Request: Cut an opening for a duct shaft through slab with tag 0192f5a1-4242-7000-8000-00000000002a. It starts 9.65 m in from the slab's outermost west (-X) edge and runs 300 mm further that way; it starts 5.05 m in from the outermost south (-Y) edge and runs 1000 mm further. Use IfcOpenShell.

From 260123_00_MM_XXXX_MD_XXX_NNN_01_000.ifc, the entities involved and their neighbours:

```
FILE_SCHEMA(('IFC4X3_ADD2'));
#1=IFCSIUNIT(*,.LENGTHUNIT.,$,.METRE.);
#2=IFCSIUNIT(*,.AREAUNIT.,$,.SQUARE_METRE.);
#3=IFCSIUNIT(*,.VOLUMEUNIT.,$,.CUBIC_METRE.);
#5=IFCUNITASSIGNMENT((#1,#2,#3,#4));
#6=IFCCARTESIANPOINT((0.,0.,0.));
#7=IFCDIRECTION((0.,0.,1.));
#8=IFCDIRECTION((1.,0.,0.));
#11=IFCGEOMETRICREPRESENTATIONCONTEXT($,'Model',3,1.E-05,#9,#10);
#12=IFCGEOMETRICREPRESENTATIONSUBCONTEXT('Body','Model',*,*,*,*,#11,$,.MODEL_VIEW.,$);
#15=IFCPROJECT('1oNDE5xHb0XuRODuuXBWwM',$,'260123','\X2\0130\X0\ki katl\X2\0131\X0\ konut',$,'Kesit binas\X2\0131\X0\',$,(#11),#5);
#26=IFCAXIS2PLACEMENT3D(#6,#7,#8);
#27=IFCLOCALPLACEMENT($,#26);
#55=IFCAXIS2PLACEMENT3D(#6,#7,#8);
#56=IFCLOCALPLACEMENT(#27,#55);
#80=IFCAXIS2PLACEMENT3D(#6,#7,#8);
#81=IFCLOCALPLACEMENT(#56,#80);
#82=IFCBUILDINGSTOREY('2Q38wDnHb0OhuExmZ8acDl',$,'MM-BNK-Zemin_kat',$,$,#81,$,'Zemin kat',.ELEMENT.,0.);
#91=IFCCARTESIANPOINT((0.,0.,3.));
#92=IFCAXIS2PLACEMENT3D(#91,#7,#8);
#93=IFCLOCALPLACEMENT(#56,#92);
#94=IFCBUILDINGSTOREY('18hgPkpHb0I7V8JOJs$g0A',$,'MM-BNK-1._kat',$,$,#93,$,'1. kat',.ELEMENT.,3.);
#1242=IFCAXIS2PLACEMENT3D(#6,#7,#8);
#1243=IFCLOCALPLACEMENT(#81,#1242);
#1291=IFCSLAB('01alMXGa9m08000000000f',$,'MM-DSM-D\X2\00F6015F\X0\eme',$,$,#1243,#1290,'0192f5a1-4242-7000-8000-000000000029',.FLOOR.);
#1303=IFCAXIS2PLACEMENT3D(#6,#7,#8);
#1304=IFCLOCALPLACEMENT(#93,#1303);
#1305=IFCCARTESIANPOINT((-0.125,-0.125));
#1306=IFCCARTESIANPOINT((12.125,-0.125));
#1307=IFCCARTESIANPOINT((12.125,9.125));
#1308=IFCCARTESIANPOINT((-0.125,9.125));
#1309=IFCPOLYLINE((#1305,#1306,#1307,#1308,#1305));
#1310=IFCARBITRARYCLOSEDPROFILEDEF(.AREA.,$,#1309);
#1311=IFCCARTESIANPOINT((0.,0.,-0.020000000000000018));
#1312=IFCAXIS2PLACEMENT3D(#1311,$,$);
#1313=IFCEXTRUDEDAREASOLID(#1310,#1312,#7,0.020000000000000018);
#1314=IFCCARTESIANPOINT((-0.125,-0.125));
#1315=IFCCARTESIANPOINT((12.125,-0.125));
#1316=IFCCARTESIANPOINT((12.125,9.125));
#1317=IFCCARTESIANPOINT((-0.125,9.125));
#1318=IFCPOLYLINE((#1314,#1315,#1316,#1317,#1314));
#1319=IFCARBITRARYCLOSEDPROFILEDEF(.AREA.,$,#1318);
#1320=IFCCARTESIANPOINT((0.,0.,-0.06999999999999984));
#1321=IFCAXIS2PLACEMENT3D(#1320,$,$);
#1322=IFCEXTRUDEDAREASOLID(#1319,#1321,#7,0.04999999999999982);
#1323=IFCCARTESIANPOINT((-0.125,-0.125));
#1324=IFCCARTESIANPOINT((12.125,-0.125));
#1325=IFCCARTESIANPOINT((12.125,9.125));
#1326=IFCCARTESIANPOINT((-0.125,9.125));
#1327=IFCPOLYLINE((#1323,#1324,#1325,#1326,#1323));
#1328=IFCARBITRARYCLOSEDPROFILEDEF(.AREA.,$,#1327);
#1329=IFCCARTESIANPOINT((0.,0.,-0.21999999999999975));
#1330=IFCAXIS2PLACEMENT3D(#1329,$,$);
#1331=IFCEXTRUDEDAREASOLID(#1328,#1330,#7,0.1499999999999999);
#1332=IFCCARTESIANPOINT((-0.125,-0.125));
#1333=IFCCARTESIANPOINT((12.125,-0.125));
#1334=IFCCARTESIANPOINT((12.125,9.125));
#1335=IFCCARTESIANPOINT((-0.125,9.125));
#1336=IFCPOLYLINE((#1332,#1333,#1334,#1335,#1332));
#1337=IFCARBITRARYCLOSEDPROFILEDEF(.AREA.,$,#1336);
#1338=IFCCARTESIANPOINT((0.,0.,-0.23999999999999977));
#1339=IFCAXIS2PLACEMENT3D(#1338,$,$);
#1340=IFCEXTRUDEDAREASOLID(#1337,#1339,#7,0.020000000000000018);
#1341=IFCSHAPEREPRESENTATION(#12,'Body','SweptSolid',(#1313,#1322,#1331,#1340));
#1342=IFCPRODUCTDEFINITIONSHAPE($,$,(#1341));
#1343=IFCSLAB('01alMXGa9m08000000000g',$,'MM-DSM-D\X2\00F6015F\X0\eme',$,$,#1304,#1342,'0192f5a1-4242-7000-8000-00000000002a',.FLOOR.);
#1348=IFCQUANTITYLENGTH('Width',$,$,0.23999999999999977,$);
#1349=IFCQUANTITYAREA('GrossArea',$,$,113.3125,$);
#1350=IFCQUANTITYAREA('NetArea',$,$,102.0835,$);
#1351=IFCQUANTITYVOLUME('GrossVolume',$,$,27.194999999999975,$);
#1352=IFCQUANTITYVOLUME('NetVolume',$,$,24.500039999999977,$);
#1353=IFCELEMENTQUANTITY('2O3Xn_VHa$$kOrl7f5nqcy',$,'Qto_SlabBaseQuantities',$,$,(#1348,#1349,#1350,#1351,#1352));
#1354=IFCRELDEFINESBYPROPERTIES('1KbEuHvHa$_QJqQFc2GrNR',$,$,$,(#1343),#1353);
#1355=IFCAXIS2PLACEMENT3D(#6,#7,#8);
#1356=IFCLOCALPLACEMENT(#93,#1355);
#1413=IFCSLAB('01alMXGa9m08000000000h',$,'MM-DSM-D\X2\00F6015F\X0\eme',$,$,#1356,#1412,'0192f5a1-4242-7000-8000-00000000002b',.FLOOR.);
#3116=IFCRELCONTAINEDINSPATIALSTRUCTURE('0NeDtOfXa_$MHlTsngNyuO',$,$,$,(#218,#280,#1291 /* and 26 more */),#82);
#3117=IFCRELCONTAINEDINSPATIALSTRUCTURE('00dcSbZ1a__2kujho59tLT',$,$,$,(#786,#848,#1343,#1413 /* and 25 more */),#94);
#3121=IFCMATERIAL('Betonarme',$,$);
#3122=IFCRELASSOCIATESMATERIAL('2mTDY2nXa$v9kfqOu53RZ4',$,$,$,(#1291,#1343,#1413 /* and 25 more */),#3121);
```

```python
import numpy as np
import ifcopenshell
import ifcopenshell.api.feature
import ifcopenshell.api.geometry
import ifcopenshell.api.pset
import ifcopenshell.api.root
import ifcopenshell.geom
import ifcopenshell.util.element
import ifcopenshell.util.placement
import ifcopenshell.util.representation
import ifcopenshell.util.shape
import ifcopenshell.util.unit

model = ifcopenshell.open("260123_00_MM_XXXX_MD_XXX_NNN_01_000.ifc")
unit_scale = ifcopenshell.util.unit.calculate_unit_scale(model)
area_scale = ifcopenshell.util.unit.calculate_unit_scale(model, "AREAUNIT")
volume_scale = ifcopenshell.util.unit.calculate_unit_scale(model, "VOLUMEUNIT")
settings = ifcopenshell.geom.settings()


def volume(element):
    """Net volume in cubic metres, openings subtracted."""
    shape = ifcopenshell.geom.create_shape(settings, element)
    return ifcopenshell.util.shape.get_volume(shape.geometry)


slab = model.by_id(1343)
before = volume(slab)

# Extent in the slab's own axes, in metres. The edges named are its -X and -Y sides.
slab_shape = ifcopenshell.geom.create_shape(settings, slab)
vertices = ifcopenshell.util.shape.get_vertices(slab_shape.geometry)
x_min, y_min, bottom = vertices.min(axis=0)
top = vertices[:, 2].max()

opening = ifcopenshell.api.root.create_entity(model, ifc_class="IfcOpeningElement", name="Duct shaft opening", predefined_type="OPENING")
context = ifcopenshell.util.representation.get_context(model, "Model", "Body", "MODEL_VIEW")
width, depth = 0.3, 1
outline = [(0.0, 0.0), (width, 0.0), (width, depth), (0.0, depth), (0.0, 0.0)]
# Overshoot both faces by 50 mm so the cut is clean.
shape = ifcopenshell.api.geometry.add_slab_representation(
    model, context=context, depth=top - bottom + 0.1, polyline=outline
)
ifcopenshell.api.geometry.assign_representation(model, product=opening, representation=shape)

matrix = ifcopenshell.util.placement.get_local_placement(slab.ObjectPlacement)
matrix[:, 3] = matrix @ np.append(np.array([x_min + 9.65, y_min + 5.05, bottom - 0.05]) / unit_scale, 1.0)
ifcopenshell.api.geometry.edit_object_placement(model, product=opening, matrix=matrix, is_si=False)
ifcopenshell.api.feature.add_feature(model, feature=opening, element=slab)

after = volume(slab)

# Update the slab's stored quantities.
qto = model.by_id(ifcopenshell.util.element.get_pset(slab, "Qto_SlabBaseQuantities", should_inherit=False)["id"])
ifcopenshell.api.pset.edit_qto(model, qto=qto, properties={
    "NetArea": after / (top - bottom) / area_scale,
    "NetVolume": after / volume_scale,
})

print(f"slab volume {before:.3f} -> {after:.3f} m3")

model.write("260123_00_MM_XXXX_MD_XXX_NNN_01_000_updated.ifc")
```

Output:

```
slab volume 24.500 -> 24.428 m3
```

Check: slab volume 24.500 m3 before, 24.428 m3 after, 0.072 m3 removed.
